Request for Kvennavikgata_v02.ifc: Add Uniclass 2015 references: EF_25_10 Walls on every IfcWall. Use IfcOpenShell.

First a look at what the model holds.

```python
import ifcopenshell

model = ifcopenshell.open("Kvennavikgata_v02.ifc")
print(model.schema)
print("classifications:", [c.Name for c in model.by_type("IfcClassification")])
for ifc_class in ("IfcDoor", "IfcRoof", "IfcStair", "IfcWall", "IfcWindow"):
    print(ifc_class, len(model.by_type(ifc_class)))
```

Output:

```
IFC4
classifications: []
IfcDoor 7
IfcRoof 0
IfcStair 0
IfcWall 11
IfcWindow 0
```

```python
import ifcopenshell
import ifcopenshell.api.classification

model = ifcopenshell.open("Kvennavikgata_v02.ifc")

system = ifcopenshell.api.classification.add_classification(model, classification="Uniclass 2015")

codes = {
    "IfcWall": ("EF_25_10", "Walls"),
}
for ifc_class, (code, name) in codes.items():
    products = model.by_type(ifc_class)
    ifcopenshell.api.classification.add_reference(
        model, products=products, classification=system, identification=code, name=name
    )
    print(code, len(products))

model.write("Kvennavikgata_v02_updated.ifc")
```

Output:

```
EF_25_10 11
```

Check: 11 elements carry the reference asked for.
